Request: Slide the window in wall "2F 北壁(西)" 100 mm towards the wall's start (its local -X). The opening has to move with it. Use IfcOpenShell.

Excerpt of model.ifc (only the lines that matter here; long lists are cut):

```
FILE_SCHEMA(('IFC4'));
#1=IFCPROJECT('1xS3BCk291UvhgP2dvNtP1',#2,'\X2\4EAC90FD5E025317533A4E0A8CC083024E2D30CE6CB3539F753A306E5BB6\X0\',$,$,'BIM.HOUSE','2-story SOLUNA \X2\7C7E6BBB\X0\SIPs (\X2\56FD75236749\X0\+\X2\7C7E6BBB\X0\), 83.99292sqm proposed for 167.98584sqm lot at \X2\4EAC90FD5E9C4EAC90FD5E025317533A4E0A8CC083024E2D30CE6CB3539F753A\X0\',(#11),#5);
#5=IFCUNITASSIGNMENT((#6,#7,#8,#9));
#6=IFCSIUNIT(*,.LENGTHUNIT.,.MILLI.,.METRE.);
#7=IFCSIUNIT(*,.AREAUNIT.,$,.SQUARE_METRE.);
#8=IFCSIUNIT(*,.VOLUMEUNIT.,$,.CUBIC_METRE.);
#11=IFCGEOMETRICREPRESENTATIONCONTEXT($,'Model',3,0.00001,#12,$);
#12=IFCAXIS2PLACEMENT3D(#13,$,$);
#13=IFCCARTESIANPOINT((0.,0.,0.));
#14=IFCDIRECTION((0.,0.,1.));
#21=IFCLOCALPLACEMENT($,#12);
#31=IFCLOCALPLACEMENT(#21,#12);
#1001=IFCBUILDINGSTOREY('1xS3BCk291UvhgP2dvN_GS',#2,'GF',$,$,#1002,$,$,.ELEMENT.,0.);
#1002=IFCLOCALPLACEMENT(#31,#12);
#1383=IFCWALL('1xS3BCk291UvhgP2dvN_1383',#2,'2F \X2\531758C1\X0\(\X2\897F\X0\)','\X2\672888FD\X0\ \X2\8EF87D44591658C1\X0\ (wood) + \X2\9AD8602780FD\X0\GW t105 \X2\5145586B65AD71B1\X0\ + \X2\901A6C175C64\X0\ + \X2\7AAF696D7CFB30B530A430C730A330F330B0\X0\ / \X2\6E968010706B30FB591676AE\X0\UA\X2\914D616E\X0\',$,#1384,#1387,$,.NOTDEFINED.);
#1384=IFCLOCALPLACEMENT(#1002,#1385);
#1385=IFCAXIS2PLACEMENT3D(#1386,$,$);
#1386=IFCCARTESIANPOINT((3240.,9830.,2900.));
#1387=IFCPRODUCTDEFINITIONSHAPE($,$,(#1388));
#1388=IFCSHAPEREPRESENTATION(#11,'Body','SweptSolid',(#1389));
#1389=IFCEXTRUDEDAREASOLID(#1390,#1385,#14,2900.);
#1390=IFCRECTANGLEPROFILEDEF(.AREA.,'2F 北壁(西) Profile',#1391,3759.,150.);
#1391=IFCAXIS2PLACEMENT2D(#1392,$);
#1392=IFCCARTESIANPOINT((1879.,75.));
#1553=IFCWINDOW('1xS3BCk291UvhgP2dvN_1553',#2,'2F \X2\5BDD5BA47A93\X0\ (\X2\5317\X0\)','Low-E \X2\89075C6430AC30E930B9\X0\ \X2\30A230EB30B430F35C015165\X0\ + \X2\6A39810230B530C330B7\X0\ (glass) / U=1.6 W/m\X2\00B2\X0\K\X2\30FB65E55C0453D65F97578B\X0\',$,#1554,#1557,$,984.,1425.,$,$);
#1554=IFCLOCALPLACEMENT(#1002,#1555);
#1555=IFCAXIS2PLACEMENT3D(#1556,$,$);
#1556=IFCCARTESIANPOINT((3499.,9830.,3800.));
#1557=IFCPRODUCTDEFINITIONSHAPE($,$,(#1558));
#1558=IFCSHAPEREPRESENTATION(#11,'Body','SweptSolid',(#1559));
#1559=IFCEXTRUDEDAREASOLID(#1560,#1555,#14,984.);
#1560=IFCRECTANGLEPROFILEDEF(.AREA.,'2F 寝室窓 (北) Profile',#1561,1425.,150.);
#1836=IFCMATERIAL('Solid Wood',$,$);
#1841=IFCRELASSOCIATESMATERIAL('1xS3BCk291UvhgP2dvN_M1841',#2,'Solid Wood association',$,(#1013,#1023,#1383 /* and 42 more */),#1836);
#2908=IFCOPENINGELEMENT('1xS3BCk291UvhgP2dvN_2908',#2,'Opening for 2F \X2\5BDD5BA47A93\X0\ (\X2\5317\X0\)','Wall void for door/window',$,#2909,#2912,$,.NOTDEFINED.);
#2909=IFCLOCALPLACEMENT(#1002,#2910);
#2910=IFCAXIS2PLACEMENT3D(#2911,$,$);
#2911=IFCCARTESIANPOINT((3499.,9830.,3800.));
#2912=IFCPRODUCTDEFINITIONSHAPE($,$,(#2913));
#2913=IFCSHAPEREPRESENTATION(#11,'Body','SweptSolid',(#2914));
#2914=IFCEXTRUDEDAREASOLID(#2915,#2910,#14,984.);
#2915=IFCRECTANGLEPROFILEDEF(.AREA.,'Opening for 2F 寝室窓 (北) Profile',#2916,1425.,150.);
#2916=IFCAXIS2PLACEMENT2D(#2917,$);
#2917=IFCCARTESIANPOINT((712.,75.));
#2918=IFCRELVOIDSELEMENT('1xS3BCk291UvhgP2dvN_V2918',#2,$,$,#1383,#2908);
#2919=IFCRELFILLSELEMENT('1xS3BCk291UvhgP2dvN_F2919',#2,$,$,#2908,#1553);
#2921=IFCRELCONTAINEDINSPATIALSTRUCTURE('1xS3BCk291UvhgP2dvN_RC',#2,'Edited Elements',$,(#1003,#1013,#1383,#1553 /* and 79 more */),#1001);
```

```python
import ifcopenshell
import ifcopenshell.api.geometry
import ifcopenshell.util.placement

model = ifcopenshell.open("model.ifc")

window = model.by_guid("1xS3BCk291UvhgP2dvN_1553")
opening = window.FillsVoids[0].RelatingOpeningElement
wall = opening.VoidsElements[0].RelatingBuildingElement

wall_matrix = ifcopenshell.util.placement.get_local_placement(wall.ObjectPlacement)
shift = wall_matrix[:3, 0] * -100.0
before = ifcopenshell.util.placement.get_local_placement(window.ObjectPlacement)[:3, 3].copy()

# The window is not placed relative to its opening, so move both.
for product in (opening, window):
    matrix = ifcopenshell.util.placement.get_local_placement(product.ObjectPlacement)
    matrix[:3, 3] += shift
    ifcopenshell.api.geometry.edit_object_placement(model, product=product, matrix=matrix, is_si=False)

after = ifcopenshell.util.placement.get_local_placement(window.ObjectPlacement)[:3, 3]
print("window moved by", (after - before).round(3) + 0.0)

model.write("model_updated.ifc")
```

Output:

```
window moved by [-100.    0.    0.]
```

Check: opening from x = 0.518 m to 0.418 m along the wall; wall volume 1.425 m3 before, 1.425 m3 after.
